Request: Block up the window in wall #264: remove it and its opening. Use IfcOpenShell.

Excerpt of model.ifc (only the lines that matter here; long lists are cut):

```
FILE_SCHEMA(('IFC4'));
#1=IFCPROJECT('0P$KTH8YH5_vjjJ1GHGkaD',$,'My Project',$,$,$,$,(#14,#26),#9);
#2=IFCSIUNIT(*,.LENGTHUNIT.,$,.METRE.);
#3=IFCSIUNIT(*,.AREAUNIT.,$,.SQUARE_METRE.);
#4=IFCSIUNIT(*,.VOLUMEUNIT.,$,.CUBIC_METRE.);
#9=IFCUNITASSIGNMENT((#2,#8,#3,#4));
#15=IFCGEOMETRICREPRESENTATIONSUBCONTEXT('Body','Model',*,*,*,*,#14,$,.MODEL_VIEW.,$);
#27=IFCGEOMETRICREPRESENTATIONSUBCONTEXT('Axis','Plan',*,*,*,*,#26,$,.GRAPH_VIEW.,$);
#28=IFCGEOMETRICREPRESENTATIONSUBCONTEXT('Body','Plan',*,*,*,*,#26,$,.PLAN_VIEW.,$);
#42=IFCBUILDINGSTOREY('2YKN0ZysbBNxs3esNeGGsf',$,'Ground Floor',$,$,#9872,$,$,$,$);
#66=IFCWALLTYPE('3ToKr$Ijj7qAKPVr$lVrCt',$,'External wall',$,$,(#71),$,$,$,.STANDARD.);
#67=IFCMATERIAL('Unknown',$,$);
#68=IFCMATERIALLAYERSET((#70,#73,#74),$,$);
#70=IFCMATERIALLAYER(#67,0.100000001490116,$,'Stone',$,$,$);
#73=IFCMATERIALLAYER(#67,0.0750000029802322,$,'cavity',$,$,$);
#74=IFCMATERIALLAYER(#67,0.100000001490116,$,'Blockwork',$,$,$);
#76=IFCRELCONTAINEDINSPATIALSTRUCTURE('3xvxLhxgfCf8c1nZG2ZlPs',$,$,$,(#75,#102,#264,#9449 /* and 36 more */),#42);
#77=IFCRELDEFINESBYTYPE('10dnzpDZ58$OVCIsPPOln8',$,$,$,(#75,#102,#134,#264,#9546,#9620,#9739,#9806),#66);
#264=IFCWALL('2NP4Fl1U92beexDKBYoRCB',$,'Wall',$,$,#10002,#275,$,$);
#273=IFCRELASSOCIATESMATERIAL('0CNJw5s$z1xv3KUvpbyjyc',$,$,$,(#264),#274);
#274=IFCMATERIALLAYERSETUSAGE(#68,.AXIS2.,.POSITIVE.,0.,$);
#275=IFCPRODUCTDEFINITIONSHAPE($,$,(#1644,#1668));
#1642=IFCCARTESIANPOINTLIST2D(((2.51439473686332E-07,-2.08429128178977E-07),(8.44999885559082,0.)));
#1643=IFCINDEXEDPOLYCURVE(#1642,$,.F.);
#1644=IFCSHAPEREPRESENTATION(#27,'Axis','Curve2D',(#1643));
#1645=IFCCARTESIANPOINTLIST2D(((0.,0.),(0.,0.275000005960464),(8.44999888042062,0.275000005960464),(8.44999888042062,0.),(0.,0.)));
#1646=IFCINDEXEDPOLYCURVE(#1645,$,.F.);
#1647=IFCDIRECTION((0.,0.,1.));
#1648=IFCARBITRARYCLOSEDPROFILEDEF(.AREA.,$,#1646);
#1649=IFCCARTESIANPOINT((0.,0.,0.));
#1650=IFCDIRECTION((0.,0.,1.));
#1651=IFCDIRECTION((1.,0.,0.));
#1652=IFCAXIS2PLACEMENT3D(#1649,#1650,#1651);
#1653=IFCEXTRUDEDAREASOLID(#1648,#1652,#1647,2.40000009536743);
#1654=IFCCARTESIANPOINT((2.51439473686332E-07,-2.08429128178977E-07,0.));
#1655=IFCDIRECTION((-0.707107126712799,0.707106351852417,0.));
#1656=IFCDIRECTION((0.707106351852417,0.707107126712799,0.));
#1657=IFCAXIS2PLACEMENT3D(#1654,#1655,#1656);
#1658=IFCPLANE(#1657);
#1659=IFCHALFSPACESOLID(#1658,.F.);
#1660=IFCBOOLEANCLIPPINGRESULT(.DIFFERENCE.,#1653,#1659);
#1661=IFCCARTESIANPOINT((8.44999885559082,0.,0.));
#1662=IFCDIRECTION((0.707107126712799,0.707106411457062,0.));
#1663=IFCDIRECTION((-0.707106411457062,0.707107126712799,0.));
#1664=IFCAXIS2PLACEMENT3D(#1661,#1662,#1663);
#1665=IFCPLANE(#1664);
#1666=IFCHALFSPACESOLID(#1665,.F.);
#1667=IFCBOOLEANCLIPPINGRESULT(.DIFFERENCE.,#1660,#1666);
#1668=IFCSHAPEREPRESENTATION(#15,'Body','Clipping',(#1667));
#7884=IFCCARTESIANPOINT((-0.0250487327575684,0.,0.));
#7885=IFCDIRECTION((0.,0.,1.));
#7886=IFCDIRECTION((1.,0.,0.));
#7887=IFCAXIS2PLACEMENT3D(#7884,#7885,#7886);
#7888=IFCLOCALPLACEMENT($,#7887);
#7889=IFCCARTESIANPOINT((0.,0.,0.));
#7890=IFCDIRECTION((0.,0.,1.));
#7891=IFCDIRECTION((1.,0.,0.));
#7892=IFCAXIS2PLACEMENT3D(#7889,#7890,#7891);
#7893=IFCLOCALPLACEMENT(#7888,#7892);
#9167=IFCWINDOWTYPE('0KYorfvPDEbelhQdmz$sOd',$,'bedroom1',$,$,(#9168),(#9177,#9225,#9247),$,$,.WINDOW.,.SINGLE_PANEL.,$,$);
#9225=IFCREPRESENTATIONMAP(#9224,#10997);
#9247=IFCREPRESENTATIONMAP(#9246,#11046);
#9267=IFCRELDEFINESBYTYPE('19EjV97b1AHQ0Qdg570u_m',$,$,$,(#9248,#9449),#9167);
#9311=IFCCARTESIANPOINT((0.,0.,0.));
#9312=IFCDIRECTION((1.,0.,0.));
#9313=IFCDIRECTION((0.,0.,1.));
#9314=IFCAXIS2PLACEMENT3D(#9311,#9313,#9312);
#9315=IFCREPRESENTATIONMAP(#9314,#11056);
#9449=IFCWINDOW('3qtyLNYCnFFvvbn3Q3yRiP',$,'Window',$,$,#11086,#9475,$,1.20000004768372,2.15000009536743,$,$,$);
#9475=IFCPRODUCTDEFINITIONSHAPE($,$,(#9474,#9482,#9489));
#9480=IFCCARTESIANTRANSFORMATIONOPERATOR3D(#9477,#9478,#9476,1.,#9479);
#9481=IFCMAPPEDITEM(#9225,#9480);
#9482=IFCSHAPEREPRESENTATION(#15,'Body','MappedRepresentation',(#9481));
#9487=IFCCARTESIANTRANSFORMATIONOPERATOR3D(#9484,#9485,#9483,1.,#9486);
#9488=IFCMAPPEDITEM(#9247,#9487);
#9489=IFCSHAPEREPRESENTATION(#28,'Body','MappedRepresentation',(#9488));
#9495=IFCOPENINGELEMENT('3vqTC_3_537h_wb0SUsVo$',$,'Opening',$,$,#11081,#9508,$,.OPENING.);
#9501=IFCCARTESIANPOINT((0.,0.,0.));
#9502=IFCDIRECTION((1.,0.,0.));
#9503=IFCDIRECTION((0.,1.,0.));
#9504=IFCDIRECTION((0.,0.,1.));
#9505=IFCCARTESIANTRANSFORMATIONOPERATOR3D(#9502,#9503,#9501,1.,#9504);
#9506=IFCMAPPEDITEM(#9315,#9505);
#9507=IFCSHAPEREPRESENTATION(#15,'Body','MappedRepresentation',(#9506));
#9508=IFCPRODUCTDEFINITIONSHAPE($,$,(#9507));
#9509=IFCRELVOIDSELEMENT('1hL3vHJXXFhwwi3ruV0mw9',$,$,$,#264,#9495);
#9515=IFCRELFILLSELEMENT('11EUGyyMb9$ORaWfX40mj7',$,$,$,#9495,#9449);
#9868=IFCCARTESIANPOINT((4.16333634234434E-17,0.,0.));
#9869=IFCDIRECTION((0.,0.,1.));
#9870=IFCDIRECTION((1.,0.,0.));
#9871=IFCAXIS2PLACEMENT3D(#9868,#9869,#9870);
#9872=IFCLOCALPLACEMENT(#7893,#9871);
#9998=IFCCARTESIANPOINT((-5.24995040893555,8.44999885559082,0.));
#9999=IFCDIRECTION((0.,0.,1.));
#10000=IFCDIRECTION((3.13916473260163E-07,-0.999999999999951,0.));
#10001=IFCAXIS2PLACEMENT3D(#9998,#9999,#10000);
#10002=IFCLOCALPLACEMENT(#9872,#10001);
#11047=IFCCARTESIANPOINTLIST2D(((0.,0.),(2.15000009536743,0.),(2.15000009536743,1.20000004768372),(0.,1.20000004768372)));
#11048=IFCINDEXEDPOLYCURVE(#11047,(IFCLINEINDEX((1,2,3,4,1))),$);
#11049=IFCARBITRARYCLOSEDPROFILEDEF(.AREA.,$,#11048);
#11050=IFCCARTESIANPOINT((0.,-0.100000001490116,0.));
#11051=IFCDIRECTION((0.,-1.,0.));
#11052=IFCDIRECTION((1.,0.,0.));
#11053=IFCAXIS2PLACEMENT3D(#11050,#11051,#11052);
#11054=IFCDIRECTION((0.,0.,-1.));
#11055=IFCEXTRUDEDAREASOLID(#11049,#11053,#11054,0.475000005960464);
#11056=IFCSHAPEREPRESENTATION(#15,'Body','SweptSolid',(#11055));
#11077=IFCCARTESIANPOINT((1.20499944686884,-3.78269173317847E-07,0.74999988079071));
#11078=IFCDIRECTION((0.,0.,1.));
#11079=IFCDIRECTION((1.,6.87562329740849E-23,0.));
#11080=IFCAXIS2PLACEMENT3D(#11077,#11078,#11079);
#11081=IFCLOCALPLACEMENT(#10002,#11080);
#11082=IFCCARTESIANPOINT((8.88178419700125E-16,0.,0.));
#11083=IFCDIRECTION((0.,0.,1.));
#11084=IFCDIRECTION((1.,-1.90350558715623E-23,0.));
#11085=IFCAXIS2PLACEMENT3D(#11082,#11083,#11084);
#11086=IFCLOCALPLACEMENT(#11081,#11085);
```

```python
import ifcopenshell
import ifcopenshell.api.feature
import ifcopenshell.api.root
import ifcopenshell.geom
import ifcopenshell.util.shape

model = ifcopenshell.open("model.ifc")
settings = ifcopenshell.geom.settings()


def volume(element):
    """Net volume in cubic metres, openings subtracted."""
    shape = ifcopenshell.geom.create_shape(settings, element)
    return ifcopenshell.util.shape.get_volume(shape.geometry)


window = model.by_guid("3qtyLNYCnFFvvbn3Q3yRiP")
opening = window.FillsVoids[0].RelatingOpeningElement
wall = opening.VoidsElements[0].RelatingBuildingElement
before = volume(wall)

ifcopenshell.api.root.remove_product(model, product=window)
ifcopenshell.api.feature.remove_feature(model, feature=opening)

after = volume(wall)

print(f"wall volume {before:.3f} -> {after:.3f} m3")

model.write("model_rev.ifc")
```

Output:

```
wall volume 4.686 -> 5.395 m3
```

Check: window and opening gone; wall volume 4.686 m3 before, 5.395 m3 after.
